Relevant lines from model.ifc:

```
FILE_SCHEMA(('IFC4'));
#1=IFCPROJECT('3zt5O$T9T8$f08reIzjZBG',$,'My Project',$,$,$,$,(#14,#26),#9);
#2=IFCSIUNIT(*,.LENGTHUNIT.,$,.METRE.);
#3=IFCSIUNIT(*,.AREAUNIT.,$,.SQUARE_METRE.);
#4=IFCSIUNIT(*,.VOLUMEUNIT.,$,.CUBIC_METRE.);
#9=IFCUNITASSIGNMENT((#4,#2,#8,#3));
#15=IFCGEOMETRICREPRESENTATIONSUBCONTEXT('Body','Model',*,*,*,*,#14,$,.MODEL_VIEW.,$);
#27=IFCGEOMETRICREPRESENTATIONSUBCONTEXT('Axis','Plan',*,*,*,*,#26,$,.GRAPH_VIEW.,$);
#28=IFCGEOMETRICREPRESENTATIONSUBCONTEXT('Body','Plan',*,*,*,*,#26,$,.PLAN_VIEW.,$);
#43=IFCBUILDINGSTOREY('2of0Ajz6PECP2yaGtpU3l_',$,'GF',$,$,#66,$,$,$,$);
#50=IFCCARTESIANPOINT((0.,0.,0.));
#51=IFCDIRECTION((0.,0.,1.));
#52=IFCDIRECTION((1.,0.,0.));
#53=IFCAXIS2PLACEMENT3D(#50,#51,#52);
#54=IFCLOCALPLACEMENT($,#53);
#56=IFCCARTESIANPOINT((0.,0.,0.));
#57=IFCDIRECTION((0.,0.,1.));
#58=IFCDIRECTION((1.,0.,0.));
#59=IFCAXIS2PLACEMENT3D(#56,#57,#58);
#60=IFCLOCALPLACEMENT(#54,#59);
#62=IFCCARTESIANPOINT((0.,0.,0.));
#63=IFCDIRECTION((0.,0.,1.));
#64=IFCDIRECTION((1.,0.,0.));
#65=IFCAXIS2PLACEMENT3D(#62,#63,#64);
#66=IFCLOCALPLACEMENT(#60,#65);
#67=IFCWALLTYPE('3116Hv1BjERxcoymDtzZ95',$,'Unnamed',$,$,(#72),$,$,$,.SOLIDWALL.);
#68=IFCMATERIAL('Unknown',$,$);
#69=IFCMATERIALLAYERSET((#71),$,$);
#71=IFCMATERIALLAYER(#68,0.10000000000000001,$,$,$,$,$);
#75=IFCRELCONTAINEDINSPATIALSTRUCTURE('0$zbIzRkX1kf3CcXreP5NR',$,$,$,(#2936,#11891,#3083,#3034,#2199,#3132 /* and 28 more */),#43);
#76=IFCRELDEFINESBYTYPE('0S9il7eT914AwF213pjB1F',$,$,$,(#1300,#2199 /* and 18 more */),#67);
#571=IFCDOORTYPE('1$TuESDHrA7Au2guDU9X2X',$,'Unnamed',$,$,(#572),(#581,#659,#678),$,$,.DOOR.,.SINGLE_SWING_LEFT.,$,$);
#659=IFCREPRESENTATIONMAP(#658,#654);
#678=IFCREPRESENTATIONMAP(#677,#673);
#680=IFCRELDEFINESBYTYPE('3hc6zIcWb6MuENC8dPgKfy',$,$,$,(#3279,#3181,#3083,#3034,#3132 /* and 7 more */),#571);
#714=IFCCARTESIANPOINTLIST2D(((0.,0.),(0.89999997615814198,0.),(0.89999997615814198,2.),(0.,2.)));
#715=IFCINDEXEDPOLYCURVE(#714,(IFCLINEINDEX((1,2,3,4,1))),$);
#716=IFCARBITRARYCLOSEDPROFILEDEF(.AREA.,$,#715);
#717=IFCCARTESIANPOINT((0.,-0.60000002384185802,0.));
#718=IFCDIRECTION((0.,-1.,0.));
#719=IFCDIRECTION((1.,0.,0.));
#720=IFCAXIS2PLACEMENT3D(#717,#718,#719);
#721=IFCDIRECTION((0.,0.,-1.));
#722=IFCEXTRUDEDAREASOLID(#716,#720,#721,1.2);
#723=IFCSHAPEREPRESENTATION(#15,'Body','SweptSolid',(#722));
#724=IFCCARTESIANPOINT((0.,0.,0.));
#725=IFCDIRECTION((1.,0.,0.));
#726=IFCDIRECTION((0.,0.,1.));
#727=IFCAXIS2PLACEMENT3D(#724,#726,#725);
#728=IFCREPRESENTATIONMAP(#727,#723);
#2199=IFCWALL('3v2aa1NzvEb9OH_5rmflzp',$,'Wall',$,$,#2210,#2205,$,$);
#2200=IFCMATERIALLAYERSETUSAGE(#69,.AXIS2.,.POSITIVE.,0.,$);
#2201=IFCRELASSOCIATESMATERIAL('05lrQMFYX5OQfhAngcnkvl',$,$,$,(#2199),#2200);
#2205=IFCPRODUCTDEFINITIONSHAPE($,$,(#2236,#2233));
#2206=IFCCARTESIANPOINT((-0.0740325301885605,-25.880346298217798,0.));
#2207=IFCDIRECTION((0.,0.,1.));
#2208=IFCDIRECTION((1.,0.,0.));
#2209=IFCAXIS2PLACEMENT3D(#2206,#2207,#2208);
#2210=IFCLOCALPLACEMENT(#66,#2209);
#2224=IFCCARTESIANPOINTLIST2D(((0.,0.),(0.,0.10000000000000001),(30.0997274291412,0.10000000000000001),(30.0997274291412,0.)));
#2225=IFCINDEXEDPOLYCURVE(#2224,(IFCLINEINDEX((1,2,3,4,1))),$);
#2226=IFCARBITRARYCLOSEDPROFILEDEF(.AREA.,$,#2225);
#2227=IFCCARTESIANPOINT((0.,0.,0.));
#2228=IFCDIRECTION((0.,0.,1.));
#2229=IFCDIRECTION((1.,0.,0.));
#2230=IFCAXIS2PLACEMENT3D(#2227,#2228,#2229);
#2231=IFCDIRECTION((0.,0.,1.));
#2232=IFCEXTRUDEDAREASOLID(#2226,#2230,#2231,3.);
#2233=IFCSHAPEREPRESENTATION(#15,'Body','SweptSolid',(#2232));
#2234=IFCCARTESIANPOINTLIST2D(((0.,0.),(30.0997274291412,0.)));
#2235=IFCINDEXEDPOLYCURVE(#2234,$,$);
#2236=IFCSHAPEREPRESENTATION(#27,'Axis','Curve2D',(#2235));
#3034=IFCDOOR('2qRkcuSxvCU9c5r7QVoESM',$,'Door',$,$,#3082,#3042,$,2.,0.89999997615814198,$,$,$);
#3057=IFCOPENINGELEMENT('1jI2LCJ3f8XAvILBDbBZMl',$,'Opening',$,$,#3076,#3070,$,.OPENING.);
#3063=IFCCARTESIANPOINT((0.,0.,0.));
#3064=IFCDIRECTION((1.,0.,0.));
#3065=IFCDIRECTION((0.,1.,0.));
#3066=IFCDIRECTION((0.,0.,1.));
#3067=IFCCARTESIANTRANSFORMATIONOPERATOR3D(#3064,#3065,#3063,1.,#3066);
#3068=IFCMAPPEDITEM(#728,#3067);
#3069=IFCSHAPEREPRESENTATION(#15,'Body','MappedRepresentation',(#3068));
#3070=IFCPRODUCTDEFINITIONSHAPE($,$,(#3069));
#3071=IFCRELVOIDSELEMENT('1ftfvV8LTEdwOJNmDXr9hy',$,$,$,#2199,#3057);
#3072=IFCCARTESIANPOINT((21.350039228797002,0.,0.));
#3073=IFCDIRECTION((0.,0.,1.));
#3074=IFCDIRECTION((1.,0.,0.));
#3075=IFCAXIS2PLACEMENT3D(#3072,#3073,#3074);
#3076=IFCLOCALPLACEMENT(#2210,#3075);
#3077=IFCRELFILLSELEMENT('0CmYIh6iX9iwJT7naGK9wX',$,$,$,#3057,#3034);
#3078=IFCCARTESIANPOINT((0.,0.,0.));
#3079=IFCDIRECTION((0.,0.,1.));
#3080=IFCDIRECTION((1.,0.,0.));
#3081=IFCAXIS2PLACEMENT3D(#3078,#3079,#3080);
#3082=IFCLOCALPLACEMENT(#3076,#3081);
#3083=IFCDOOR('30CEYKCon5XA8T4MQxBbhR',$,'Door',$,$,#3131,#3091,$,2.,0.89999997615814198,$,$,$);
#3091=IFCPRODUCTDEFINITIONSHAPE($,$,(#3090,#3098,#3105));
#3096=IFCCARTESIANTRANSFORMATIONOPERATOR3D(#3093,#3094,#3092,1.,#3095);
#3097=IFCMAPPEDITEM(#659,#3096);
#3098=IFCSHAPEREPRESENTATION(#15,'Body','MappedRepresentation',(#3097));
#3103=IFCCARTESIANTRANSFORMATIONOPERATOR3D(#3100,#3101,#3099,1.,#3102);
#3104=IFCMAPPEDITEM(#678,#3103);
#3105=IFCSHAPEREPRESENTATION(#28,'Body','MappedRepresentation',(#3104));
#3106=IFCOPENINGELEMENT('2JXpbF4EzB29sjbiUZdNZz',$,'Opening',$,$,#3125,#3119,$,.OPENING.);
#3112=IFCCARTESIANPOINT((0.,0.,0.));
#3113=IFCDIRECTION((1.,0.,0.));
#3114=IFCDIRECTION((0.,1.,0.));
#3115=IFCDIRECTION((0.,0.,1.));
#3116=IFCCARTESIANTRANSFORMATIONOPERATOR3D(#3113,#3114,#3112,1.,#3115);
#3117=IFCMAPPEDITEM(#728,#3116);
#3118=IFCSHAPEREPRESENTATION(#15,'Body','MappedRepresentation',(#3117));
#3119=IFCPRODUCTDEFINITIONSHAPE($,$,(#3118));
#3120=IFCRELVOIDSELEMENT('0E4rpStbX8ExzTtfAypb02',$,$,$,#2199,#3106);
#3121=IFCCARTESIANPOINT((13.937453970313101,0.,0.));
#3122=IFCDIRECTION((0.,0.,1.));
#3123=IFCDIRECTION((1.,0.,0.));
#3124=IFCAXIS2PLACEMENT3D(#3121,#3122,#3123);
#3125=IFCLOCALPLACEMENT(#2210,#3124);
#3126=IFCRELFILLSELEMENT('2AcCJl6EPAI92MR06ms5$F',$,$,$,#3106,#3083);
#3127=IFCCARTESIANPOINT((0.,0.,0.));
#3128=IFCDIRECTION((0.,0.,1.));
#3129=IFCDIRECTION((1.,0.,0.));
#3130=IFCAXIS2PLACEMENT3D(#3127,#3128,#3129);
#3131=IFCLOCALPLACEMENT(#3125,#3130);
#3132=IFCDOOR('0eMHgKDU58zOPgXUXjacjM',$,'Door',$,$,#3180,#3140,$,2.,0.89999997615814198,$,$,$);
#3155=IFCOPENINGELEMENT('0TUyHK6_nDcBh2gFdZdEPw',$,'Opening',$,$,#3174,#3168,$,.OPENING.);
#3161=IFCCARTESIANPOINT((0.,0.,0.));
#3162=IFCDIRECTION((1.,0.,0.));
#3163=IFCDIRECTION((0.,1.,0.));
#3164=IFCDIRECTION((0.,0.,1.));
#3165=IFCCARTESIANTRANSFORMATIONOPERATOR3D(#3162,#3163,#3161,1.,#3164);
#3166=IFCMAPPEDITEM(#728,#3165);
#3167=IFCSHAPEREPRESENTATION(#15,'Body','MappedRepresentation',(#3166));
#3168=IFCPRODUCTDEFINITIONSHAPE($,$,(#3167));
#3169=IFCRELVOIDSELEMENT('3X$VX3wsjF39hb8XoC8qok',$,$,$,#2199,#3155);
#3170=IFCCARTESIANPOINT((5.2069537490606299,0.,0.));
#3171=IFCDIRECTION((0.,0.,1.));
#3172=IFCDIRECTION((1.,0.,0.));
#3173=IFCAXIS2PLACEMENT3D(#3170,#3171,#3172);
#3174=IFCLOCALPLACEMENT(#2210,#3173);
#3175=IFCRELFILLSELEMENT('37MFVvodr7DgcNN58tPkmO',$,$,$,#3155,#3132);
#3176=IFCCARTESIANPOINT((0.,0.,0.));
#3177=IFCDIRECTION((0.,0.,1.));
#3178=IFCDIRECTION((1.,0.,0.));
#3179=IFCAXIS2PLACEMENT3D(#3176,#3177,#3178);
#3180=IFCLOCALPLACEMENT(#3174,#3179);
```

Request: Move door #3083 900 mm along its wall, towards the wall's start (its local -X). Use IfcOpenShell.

```python
import ifcopenshell
import ifcopenshell.api.geometry
import ifcopenshell.util.placement
import ifcopenshell.util.unit

model = ifcopenshell.open("model.ifc")
unit_scale = ifcopenshell.util.unit.calculate_unit_scale(model)

door = model.by_id(3083)
opening = door.FillsVoids[0].RelatingOpeningElement
wall = opening.VoidsElements[0].RelatingBuildingElement

wall_matrix = ifcopenshell.util.placement.get_local_placement(wall.ObjectPlacement)
shift = wall_matrix[:3, 0] * -0.9 / unit_scale
before = ifcopenshell.util.placement.get_local_placement(door.ObjectPlacement)[:3, 3].copy()

# The door is placed relative to its opening, so it follows when the opening moves.
matrix = ifcopenshell.util.placement.get_local_placement(opening.ObjectPlacement)
matrix[:3, 3] += shift
ifcopenshell.api.geometry.edit_object_placement(
    model, product=opening, matrix=matrix, is_si=False, should_transform_children=True
)

after = ifcopenshell.util.placement.get_local_placement(door.ObjectPlacement)[:3, 3]
print("door moved by", (after - before).round(3) + 0.0)

model.write("model_v2.ifc")
```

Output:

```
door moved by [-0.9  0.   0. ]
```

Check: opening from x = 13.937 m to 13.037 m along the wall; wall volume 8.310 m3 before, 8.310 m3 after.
